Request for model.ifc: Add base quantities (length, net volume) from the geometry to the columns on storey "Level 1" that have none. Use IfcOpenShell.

First a look at what the model holds.

```python
import ifcopenshell
import ifcopenshell.util.element
import ifcopenshell.util.unit

model = ifcopenshell.open("model.ifc")
print(model.schema)
for unit_type in ("LENGTHUNIT", "AREAUNIT", "VOLUMEUNIT"):
    print(unit_type, ifcopenshell.util.unit.calculate_unit_scale(model, unit_type))
storey = next(s for s in model.by_type("IfcBuildingStorey") if s.Name == "Level 1")
columns = [e for e in ifcopenshell.util.element.get_decomposition(storey) if e.is_a("IfcColumn")]
for e in sorted(columns, key=lambda e: e.id()):
    print(e.id(), e.is_a(), e.Name, list(ifcopenshell.util.element.get_psets(e, qtos_only=True)), sep=" | ")
```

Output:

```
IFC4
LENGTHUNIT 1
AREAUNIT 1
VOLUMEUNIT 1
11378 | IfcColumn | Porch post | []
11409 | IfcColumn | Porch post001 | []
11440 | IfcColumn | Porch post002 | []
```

```python
import ifcopenshell
import ifcopenshell.api.pset
import ifcopenshell.geom
import ifcopenshell.util.element
import ifcopenshell.util.shape
import ifcopenshell.util.unit

model = ifcopenshell.open("model.ifc")
unit_scale = ifcopenshell.util.unit.calculate_unit_scale(model)
volume_scale = ifcopenshell.util.unit.calculate_unit_scale(model, "VOLUMEUNIT")
settings = ifcopenshell.geom.settings()

storey = next(s for s in model.by_type("IfcBuildingStorey") if s.Name == "Level 1")
columns = [e for e in ifcopenshell.util.element.get_decomposition(storey) if e.is_a("IfcColumn")]

for e in sorted(columns, key=lambda e: e.id()):
    if ifcopenshell.util.element.get_psets(e, qtos_only=True, should_inherit=False):
        continue
    # Geometry comes back in metres, in the element's own axes.
    shape = ifcopenshell.geom.create_shape(settings, e)
    values = {
        "Length": ifcopenshell.util.shape.get_z(shape.geometry) / unit_scale,
        "NetVolume": ifcopenshell.util.shape.get_volume(shape.geometry) / volume_scale,
    }
    qto = ifcopenshell.api.pset.add_qto(model, product=e, name="Qto_ColumnBaseQuantities")
    ifcopenshell.api.pset.edit_qto(model, qto=qto, properties=values)
    print(e.id(), {k: round(v, 3) for k, v in values.items()})

model.write("model_rev.ifc")
```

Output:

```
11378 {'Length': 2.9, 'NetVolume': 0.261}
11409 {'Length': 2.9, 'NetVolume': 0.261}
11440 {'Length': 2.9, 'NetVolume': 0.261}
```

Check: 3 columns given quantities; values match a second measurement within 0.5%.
